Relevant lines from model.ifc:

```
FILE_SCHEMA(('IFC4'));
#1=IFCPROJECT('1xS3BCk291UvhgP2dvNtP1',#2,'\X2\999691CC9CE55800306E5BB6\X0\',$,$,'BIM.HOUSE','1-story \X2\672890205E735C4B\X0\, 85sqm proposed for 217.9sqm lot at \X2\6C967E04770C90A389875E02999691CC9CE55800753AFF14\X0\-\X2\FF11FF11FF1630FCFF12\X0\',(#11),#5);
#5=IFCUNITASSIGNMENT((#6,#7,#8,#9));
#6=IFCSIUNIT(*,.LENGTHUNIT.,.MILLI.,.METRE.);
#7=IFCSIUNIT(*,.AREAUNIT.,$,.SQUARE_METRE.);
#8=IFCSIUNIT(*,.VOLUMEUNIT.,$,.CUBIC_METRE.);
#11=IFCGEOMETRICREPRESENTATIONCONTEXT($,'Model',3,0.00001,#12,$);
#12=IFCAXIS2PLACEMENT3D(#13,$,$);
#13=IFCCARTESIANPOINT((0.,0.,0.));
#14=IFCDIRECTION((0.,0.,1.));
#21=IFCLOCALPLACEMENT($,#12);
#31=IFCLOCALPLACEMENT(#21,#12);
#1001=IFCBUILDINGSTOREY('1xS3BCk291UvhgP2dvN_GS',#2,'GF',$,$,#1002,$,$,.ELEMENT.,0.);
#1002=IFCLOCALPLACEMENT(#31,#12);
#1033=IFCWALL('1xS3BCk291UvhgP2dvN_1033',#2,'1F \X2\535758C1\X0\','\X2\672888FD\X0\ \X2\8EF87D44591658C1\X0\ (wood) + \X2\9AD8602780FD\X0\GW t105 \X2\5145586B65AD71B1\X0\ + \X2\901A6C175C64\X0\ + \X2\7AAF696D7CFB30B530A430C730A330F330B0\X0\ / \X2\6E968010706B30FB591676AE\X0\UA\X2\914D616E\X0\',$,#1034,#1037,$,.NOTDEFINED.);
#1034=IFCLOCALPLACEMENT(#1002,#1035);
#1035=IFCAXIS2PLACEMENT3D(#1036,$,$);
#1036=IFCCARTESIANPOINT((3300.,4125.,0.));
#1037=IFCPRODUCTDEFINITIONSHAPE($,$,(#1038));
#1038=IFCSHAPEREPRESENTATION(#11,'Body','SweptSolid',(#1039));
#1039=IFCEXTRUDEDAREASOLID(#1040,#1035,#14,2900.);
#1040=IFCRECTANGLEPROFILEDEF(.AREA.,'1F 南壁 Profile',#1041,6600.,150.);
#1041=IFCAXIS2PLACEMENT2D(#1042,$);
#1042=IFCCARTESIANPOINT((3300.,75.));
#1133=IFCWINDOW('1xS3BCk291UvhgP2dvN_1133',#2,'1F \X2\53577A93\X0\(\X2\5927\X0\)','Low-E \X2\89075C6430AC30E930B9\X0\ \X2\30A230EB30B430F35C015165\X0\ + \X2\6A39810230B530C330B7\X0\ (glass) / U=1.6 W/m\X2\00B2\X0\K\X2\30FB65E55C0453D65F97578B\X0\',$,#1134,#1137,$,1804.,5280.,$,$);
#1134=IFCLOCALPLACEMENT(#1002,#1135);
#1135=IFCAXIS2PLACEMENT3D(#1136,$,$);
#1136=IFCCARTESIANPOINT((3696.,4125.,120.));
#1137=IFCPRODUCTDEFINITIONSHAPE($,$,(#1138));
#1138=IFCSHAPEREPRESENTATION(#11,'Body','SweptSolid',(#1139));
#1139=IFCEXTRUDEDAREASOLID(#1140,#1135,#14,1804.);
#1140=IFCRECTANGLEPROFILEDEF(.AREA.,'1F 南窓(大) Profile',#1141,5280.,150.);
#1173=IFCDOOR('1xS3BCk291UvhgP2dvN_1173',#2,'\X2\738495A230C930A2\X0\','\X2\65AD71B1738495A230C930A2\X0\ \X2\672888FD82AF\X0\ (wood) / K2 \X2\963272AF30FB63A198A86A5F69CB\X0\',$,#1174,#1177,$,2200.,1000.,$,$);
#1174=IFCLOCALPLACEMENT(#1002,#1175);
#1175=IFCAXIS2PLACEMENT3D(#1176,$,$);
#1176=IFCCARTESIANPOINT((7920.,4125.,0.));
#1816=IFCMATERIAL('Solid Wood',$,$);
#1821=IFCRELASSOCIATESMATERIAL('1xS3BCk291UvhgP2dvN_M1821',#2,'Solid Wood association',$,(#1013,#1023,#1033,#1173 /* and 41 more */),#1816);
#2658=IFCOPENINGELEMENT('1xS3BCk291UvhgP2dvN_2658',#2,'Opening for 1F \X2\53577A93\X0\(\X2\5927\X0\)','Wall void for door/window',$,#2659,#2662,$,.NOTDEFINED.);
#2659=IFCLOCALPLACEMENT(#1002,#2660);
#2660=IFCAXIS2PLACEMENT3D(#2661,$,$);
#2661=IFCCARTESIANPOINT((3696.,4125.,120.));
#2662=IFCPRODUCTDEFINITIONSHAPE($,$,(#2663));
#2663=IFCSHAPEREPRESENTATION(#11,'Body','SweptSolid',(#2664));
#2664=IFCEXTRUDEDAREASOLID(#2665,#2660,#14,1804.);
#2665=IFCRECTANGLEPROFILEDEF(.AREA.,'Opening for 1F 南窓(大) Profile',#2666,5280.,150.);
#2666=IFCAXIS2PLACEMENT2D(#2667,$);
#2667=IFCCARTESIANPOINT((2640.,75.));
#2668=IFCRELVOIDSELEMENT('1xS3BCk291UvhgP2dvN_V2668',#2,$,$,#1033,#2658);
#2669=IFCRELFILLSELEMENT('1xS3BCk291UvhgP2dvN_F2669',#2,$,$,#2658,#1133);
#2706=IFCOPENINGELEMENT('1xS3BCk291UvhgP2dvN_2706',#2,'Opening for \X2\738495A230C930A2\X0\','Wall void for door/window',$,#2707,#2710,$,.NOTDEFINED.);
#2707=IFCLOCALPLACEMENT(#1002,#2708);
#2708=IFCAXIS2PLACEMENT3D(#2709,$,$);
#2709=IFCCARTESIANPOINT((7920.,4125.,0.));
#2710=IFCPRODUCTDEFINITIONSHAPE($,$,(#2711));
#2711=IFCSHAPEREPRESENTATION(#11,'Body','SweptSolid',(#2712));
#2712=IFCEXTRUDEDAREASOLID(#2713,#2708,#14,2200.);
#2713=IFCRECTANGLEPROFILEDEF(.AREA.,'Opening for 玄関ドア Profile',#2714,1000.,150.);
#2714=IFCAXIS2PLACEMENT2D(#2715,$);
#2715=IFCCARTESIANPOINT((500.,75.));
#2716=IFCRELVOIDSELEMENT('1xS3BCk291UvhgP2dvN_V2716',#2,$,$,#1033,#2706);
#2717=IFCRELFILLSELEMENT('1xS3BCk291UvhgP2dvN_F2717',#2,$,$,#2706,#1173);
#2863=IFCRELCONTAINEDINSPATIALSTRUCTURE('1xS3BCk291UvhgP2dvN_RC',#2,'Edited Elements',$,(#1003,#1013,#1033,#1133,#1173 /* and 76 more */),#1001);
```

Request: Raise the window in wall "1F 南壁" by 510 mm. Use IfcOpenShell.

```python
import numpy as np
import ifcopenshell
import ifcopenshell.api.geometry
import ifcopenshell.util.placement
import ifcopenshell.util.unit

model = ifcopenshell.open("model.ifc")
unit_scale = ifcopenshell.util.unit.calculate_unit_scale(model)

window = model.by_guid("1xS3BCk291UvhgP2dvN_1133")
opening = window.FillsVoids[0].RelatingOpeningElement
dz = 0.51 / unit_scale

shift = np.array([0.0, 0.0, dz])
# The window is not placed relative to its opening, so move both.
for product in (opening, window):
    matrix = ifcopenshell.util.placement.get_local_placement(product.ObjectPlacement)
    matrix[:3, 3] += shift
    ifcopenshell.api.geometry.edit_object_placement(model, product=product, matrix=matrix, is_si=False)

print(f"moved by {dz * unit_scale:+.3f} m")

model.write("model_rev.ifc")
```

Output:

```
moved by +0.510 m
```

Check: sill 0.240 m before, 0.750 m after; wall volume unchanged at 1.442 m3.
